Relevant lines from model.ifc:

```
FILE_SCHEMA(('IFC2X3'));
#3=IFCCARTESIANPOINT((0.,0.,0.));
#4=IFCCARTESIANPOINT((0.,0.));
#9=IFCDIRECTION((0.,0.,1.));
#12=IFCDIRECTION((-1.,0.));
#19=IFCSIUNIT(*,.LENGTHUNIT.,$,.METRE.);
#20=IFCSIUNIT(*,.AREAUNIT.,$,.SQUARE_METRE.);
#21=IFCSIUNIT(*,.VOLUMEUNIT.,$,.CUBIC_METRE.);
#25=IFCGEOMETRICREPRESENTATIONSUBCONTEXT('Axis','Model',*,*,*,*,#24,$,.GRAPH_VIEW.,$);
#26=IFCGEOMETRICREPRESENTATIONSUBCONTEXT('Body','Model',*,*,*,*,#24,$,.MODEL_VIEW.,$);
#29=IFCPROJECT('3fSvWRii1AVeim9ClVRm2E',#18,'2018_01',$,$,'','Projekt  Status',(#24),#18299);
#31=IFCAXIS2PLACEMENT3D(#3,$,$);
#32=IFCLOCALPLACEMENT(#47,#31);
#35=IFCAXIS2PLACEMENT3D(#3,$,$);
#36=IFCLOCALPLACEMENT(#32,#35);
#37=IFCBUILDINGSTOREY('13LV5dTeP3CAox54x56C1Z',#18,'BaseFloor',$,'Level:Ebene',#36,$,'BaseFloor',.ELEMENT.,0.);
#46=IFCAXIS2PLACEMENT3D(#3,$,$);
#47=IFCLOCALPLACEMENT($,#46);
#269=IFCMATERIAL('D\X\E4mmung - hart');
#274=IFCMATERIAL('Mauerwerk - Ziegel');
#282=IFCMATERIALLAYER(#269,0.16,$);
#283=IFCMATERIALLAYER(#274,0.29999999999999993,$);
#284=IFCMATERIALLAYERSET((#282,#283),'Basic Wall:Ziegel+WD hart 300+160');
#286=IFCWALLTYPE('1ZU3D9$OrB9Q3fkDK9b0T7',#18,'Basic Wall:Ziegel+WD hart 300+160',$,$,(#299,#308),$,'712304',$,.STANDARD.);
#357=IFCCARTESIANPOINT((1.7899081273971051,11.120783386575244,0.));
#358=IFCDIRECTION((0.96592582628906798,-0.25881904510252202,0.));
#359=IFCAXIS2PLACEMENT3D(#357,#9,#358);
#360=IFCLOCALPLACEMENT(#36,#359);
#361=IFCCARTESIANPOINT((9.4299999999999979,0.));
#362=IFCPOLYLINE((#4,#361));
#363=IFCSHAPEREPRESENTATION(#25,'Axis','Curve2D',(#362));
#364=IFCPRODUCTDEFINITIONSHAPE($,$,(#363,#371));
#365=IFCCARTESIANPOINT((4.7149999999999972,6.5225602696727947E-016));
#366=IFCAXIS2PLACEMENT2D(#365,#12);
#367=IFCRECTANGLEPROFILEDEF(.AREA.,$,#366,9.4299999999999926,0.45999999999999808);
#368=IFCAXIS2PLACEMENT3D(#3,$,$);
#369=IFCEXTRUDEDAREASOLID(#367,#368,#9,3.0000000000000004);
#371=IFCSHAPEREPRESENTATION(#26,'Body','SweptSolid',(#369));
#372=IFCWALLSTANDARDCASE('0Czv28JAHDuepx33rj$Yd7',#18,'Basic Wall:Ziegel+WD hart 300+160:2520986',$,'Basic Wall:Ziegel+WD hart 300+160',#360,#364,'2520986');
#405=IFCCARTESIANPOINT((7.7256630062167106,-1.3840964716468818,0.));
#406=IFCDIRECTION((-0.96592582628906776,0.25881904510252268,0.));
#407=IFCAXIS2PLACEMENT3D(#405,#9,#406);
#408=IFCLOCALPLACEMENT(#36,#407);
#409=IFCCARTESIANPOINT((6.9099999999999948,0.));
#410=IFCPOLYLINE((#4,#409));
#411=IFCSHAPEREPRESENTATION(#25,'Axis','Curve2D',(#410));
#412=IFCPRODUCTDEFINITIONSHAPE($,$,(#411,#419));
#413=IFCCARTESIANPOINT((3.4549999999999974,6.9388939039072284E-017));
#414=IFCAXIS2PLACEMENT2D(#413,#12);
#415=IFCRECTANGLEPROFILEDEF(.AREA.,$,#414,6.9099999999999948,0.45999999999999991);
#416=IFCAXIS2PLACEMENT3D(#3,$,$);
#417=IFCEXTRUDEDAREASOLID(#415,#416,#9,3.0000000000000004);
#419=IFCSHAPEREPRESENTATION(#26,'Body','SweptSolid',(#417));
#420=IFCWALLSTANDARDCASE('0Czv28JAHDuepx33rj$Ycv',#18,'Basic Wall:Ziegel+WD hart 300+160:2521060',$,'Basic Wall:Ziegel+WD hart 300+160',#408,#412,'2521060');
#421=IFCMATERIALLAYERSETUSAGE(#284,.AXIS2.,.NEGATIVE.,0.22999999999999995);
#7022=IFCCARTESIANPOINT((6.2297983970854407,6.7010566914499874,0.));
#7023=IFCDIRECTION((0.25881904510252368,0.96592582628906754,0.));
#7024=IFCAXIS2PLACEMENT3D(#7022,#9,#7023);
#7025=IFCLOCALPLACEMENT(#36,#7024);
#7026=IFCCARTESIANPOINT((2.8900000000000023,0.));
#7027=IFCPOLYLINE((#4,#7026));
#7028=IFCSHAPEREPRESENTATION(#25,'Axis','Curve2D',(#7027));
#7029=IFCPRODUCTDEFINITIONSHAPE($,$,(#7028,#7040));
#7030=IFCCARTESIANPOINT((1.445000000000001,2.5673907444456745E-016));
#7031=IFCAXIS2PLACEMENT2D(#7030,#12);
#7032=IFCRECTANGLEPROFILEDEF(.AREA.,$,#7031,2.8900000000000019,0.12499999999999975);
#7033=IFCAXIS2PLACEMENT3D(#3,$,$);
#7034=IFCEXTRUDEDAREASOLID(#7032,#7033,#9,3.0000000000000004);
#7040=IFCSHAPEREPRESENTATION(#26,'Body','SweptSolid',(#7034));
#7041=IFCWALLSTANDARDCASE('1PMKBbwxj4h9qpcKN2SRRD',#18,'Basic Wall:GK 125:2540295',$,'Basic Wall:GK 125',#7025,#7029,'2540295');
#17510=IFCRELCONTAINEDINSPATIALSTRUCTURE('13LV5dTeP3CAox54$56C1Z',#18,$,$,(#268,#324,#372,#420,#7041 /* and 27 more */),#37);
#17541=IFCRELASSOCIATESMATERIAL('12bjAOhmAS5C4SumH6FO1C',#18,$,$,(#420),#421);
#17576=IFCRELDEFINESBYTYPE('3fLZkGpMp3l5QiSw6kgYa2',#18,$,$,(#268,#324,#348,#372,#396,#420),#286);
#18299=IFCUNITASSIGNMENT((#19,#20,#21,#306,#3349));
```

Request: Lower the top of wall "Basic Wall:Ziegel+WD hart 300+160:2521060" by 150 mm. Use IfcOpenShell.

```python
import ifcopenshell
import ifcopenshell.geom
import ifcopenshell.util.representation
import ifcopenshell.util.shape
import ifcopenshell.util.unit

model = ifcopenshell.open("model.ifc")
unit_scale = ifcopenshell.util.unit.calculate_unit_scale(model)
settings = ifcopenshell.geom.settings()


def volume(element):
    """Net volume in cubic metres, openings subtracted."""
    shape = ifcopenshell.geom.create_shape(settings, element)
    return ifcopenshell.util.shape.get_volume(shape.geometry)


wall = model.by_id(420)
before = volume(wall)

body = ifcopenshell.util.representation.get_representation(wall, "Model", "Body")
solid = body.Items[0]
old_height = solid.Depth
solid.Depth -= 0.15 / unit_scale
after = volume(wall)

print(f"height {old_height:g} -> {solid.Depth:g}, volume {before:.3f} -> {after:.3f} m3")

model.write("model_edited.ifc")
```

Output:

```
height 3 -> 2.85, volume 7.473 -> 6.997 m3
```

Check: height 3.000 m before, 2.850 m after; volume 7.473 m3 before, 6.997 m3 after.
